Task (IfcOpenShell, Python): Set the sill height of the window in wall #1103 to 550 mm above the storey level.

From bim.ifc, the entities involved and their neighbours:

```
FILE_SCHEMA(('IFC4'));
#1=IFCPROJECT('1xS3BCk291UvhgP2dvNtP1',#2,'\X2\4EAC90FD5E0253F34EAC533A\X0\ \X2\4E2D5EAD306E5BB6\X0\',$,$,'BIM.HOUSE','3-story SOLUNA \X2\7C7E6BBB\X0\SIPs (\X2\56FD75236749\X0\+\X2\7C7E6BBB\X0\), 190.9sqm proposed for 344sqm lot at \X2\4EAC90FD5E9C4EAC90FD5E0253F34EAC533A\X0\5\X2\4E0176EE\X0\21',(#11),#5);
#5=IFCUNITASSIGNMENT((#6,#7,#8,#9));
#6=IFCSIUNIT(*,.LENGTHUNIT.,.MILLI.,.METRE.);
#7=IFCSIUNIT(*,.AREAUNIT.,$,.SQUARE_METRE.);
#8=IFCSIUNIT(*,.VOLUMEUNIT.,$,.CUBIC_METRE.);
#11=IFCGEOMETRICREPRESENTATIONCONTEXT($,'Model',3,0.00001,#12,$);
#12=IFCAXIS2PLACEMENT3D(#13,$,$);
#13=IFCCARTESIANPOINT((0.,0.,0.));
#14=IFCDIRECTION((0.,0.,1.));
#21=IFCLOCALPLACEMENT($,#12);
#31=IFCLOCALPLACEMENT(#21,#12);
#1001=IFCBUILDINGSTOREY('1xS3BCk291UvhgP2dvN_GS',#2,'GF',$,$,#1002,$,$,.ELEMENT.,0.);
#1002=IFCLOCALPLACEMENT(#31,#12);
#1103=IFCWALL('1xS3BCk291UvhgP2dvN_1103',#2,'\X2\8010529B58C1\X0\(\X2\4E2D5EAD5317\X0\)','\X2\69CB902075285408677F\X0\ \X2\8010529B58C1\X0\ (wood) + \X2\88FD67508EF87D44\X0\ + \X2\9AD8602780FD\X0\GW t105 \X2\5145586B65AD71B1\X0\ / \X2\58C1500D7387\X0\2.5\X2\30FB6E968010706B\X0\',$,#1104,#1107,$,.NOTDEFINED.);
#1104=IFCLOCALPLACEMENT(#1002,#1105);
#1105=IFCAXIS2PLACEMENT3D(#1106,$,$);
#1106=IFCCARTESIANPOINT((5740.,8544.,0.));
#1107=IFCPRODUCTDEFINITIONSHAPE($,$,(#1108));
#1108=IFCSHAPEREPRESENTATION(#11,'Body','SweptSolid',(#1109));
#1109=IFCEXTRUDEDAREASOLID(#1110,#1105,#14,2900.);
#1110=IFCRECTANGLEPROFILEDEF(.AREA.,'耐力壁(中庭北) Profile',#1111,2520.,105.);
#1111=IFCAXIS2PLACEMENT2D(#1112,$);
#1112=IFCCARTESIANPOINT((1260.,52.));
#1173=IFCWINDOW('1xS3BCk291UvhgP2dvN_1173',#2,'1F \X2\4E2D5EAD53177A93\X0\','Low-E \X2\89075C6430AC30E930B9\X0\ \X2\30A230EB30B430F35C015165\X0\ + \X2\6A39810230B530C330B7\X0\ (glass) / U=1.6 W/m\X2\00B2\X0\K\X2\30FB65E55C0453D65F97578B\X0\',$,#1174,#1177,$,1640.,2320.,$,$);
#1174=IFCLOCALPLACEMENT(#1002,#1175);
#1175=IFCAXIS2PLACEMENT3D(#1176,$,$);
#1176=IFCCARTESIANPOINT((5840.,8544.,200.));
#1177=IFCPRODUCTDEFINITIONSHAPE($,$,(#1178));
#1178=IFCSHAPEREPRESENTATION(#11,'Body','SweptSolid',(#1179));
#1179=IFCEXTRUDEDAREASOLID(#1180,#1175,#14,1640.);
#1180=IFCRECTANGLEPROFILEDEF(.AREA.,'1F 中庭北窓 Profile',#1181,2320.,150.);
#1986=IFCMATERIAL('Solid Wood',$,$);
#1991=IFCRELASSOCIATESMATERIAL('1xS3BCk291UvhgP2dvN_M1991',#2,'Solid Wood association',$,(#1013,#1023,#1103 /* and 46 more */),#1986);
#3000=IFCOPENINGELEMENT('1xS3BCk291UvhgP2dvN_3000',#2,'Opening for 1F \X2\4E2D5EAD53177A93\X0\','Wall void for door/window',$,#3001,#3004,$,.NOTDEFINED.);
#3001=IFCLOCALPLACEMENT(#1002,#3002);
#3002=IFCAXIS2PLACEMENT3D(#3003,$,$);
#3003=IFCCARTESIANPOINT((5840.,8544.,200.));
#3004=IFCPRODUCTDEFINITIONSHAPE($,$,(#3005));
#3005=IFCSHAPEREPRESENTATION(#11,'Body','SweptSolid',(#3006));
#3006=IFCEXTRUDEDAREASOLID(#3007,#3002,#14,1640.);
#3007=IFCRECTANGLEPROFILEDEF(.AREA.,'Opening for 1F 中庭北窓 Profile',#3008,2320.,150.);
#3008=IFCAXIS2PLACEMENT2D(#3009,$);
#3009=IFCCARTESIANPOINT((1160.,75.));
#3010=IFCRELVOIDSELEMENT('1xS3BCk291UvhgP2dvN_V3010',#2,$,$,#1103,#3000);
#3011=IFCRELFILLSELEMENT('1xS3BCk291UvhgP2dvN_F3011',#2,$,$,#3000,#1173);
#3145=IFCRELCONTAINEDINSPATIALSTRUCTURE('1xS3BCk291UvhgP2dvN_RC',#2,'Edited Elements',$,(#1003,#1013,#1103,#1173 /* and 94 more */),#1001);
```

```python
import numpy as np
import ifcopenshell
import ifcopenshell.api.geometry
import ifcopenshell.geom
import ifcopenshell.util.element
import ifcopenshell.util.placement
import ifcopenshell.util.shape
import ifcopenshell.util.unit

model = ifcopenshell.open("bim.ifc")
unit_scale = ifcopenshell.util.unit.calculate_unit_scale(model)

window = model.by_id(1173)
opening = window.FillsVoids[0].RelatingOpeningElement
storey = ifcopenshell.util.element.get_container(window, ifc_class="IfcBuildingStorey")
level = ifcopenshell.util.placement.get_local_placement(storey.ObjectPlacement)[2, 3]

# The opening's origin need not be at the sill, so measure its lowest point.
shape = ifcopenshell.geom.create_shape(ifcopenshell.geom.settings(), opening)
bottom = ifcopenshell.util.shape.get_shape_bottom_elevation(shape, shape.geometry) / unit_scale
dz = level + 0.55 / unit_scale - bottom

shift = np.array([0.0, 0.0, dz])
# The window is not placed relative to its opening, so move both.
for product in (opening, window):
    matrix = ifcopenshell.util.placement.get_local_placement(product.ObjectPlacement)
    matrix[:3, 3] += shift
    ifcopenshell.api.geometry.edit_object_placement(model, product=product, matrix=matrix, is_si=False)

print(f"moved by {dz * unit_scale:+.3f} m")

model.write("bim_rev.ifc")
```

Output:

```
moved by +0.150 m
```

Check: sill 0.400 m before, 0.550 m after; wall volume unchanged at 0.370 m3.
